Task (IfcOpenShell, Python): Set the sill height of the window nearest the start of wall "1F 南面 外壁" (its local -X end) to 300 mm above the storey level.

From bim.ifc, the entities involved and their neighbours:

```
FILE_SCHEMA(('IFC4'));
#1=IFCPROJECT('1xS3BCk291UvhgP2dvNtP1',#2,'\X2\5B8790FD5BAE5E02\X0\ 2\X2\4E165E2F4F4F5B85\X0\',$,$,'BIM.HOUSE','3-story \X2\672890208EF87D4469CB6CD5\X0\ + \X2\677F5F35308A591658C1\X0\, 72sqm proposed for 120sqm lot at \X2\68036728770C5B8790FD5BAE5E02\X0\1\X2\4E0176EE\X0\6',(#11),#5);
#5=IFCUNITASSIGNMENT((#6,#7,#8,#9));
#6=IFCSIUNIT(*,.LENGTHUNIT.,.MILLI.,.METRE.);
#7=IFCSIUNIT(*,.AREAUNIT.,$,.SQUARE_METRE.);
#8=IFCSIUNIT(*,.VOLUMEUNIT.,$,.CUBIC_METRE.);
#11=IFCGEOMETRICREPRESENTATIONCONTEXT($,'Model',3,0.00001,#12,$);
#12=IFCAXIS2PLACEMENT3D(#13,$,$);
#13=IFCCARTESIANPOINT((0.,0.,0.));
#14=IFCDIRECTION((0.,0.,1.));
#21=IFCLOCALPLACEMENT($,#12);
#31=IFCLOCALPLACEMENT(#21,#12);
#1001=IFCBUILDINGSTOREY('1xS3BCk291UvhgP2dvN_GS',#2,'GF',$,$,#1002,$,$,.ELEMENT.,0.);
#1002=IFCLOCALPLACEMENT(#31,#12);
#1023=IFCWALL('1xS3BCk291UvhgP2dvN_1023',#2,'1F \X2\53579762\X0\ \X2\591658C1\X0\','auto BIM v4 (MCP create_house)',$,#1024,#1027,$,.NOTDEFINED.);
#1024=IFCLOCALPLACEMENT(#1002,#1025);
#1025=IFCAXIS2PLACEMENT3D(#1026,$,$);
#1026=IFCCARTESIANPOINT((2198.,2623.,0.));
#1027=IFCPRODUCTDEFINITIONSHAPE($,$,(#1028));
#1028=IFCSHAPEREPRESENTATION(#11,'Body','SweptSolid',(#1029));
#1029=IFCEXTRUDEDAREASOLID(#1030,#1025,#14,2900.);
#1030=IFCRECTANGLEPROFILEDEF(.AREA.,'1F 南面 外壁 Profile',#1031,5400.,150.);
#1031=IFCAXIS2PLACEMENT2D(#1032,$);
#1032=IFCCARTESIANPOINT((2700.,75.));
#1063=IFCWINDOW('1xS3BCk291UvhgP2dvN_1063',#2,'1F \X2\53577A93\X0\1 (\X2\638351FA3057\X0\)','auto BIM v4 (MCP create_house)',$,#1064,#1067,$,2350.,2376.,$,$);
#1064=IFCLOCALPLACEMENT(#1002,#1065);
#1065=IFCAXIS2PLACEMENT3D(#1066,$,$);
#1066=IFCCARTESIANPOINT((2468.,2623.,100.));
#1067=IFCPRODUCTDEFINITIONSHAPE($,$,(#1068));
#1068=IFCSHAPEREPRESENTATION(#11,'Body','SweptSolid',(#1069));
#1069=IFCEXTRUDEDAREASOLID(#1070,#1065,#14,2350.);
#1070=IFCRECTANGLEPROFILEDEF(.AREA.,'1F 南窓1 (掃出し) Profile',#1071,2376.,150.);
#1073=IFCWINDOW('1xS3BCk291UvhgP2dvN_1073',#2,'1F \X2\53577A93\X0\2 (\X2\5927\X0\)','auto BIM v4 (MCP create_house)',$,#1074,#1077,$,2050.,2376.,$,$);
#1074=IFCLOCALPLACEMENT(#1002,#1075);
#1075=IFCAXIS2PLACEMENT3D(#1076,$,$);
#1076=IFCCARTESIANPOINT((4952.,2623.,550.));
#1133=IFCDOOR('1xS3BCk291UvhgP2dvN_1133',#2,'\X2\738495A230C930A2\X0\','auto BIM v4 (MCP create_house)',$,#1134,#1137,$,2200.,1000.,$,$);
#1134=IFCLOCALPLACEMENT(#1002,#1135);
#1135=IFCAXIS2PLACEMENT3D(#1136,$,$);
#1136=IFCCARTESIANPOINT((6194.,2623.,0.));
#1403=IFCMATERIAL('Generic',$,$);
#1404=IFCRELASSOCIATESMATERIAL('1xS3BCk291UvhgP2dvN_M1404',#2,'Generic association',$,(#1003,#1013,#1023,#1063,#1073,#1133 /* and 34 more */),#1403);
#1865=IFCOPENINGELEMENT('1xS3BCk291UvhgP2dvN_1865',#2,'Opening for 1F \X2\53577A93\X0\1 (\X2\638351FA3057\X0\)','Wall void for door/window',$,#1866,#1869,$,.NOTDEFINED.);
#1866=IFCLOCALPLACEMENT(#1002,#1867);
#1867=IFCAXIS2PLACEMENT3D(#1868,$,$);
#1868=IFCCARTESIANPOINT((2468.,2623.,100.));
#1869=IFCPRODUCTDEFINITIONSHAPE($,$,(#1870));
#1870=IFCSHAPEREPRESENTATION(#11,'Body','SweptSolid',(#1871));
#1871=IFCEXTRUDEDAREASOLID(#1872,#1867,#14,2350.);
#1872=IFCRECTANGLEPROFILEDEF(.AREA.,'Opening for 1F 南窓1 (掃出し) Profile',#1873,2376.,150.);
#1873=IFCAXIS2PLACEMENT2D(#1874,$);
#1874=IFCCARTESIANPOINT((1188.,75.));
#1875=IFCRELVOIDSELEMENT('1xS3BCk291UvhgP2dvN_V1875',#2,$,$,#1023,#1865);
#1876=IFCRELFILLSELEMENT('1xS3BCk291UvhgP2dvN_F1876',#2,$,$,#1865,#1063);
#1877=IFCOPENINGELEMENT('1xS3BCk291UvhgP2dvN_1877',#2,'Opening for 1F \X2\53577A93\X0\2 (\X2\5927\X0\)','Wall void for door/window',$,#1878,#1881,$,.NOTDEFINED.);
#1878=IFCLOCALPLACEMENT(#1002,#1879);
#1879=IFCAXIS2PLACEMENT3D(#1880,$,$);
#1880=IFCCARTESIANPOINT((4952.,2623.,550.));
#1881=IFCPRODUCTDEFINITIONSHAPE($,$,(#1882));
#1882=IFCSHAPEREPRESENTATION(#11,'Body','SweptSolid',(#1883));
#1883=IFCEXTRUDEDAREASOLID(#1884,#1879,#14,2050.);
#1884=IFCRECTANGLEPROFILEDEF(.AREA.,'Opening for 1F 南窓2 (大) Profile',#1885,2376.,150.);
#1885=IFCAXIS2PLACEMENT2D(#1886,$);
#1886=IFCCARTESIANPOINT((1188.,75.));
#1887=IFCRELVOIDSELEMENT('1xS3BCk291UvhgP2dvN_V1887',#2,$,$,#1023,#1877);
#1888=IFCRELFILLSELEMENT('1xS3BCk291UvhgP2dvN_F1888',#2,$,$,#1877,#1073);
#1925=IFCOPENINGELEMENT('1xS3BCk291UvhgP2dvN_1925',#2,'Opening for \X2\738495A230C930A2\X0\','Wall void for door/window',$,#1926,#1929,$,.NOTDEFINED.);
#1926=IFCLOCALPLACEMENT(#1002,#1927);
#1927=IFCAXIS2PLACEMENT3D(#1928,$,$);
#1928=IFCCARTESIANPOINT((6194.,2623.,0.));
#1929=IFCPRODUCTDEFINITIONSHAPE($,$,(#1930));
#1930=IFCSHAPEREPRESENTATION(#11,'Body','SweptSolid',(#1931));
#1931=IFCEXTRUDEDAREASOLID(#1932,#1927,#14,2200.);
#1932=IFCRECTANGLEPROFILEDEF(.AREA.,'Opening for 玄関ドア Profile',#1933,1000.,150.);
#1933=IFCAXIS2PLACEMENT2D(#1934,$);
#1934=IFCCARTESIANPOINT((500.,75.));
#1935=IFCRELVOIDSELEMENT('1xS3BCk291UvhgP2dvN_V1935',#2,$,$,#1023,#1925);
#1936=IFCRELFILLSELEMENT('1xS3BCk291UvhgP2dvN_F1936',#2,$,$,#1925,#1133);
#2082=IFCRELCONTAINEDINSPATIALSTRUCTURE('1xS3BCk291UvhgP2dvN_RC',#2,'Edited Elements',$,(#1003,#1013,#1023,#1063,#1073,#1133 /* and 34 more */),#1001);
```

```python
import numpy as np
import ifcopenshell
import ifcopenshell.api.geometry
import ifcopenshell.geom
import ifcopenshell.util.element
import ifcopenshell.util.placement
import ifcopenshell.util.shape
import ifcopenshell.util.unit

model = ifcopenshell.open("bim.ifc")
unit_scale = ifcopenshell.util.unit.calculate_unit_scale(model)

window = model.by_guid("1xS3BCk291UvhgP2dvN_1063")
opening = window.FillsVoids[0].RelatingOpeningElement
storey = ifcopenshell.util.element.get_container(window, ifc_class="IfcBuildingStorey")
level = ifcopenshell.util.placement.get_local_placement(storey.ObjectPlacement)[2, 3]

# The opening's origin need not be at the sill, so measure its lowest point.
shape = ifcopenshell.geom.create_shape(ifcopenshell.geom.settings(), opening)
bottom = ifcopenshell.util.shape.get_shape_bottom_elevation(shape, shape.geometry) / unit_scale
dz = level + 0.3 / unit_scale - bottom

shift = np.array([0.0, 0.0, dz])
# The window is not placed relative to its opening, so move both.
for product in (opening, window):
    matrix = ifcopenshell.util.placement.get_local_placement(product.ObjectPlacement)
    matrix[:3, 3] += shift
    ifcopenshell.api.geometry.edit_object_placement(model, product=product, matrix=matrix, is_si=False)

print(f"moved by {dz * unit_scale:+.3f} m")

model.write("bim_v2.ifc")
```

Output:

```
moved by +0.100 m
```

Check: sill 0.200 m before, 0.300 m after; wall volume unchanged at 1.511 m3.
